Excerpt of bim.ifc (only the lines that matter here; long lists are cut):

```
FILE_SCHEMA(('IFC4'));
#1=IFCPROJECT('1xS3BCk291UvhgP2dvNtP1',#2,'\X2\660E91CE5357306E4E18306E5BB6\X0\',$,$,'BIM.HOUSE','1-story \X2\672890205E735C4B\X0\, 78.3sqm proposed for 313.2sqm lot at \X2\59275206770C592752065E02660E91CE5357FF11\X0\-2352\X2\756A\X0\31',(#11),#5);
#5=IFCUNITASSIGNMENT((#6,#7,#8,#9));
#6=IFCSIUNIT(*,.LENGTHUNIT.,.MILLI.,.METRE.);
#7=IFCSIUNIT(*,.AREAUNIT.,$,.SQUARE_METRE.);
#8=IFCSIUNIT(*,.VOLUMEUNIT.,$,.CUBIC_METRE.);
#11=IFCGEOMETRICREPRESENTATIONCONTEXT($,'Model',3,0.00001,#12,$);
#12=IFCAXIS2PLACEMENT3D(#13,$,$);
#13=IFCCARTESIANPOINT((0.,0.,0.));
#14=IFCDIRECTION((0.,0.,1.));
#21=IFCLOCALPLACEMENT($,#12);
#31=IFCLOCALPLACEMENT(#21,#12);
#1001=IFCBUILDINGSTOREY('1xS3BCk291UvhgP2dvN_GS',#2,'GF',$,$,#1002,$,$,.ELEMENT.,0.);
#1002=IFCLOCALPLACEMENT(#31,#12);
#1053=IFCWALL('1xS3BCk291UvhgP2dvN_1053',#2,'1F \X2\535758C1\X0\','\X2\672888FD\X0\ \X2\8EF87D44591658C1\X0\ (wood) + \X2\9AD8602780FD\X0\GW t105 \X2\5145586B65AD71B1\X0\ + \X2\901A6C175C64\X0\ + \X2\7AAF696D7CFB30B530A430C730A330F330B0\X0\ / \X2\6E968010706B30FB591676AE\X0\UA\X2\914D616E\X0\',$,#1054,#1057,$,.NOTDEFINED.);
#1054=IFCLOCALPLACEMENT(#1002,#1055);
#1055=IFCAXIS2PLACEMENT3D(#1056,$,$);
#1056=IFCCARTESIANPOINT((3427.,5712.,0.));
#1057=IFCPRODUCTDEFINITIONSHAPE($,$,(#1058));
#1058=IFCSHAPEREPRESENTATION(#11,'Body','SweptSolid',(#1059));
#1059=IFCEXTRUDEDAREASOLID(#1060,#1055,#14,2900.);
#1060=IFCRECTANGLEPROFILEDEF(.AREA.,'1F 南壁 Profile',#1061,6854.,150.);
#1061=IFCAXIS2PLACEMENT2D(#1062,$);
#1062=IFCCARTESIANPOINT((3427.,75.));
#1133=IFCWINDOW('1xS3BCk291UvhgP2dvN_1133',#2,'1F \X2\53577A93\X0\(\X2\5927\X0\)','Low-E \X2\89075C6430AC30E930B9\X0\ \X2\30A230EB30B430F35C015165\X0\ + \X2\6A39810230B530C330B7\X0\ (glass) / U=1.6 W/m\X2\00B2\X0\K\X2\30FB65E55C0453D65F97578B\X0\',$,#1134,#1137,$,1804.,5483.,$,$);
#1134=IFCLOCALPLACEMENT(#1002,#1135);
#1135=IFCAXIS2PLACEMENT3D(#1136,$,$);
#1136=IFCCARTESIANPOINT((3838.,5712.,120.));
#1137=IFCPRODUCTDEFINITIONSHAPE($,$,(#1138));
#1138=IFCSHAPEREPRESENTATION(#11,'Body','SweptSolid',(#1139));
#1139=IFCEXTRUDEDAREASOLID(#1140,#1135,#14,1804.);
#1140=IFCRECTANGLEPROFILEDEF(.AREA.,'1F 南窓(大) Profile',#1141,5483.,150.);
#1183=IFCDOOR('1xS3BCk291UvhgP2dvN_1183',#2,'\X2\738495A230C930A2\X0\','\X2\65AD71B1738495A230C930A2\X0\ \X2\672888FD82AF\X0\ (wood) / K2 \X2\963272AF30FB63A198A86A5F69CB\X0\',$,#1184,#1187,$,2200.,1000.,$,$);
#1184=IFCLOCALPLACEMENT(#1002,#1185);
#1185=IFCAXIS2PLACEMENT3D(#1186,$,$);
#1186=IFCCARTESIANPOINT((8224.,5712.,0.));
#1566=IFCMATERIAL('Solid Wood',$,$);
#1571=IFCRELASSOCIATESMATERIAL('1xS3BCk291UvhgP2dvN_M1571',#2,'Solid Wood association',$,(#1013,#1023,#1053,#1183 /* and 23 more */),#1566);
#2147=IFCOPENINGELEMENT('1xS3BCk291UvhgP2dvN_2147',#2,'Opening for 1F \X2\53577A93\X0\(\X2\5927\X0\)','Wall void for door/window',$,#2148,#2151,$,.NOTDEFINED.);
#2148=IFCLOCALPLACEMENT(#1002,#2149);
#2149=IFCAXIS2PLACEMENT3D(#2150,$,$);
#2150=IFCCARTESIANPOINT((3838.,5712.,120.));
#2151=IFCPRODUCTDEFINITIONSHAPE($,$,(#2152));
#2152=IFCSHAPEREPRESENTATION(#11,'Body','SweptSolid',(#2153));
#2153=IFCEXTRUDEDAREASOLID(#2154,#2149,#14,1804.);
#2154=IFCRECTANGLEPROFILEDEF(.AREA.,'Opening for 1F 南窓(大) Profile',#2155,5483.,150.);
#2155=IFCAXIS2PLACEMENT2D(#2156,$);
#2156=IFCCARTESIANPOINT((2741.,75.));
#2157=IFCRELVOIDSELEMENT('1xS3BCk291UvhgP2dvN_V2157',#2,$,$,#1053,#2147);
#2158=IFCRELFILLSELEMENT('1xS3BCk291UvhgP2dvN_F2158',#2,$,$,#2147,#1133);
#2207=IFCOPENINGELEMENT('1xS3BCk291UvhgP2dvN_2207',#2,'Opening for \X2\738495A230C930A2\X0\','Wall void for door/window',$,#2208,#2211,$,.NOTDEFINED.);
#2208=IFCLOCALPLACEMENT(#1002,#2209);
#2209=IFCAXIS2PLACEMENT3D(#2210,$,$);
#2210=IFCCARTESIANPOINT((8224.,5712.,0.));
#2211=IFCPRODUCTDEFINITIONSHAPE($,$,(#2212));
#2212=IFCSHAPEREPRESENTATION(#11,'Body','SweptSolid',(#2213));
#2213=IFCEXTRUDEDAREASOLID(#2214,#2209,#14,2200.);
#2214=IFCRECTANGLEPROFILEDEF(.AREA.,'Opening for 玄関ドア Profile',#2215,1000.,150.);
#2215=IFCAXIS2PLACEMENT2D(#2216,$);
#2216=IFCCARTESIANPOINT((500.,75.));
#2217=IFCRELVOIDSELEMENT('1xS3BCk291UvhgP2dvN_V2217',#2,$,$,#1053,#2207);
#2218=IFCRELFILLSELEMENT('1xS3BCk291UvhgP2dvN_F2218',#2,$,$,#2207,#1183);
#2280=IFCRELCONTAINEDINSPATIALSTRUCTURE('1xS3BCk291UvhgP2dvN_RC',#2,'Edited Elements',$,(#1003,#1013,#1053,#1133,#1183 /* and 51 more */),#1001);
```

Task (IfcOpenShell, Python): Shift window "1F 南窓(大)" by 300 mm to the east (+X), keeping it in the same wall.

```python
import ifcopenshell
import ifcopenshell.api.geometry
import ifcopenshell.util.placement
import ifcopenshell.util.unit

model = ifcopenshell.open("bim.ifc")
unit_scale = ifcopenshell.util.unit.calculate_unit_scale(model)

window = model.by_guid("1xS3BCk291UvhgP2dvN_1133")
opening = window.FillsVoids[0].RelatingOpeningElement
wall = opening.VoidsElements[0].RelatingBuildingElement

wall_matrix = ifcopenshell.util.placement.get_local_placement(wall.ObjectPlacement)
shift = wall_matrix[:3, 0] * 0.3 / unit_scale
before = ifcopenshell.util.placement.get_local_placement(window.ObjectPlacement)[:3, 3].copy()

# The window is not placed relative to its opening, so move both.
for product in (opening, window):
    matrix = ifcopenshell.util.placement.get_local_placement(product.ObjectPlacement)
    matrix[:3, 3] += shift
    ifcopenshell.api.geometry.edit_object_placement(model, product=product, matrix=matrix, is_si=False)

after = ifcopenshell.util.placement.get_local_placement(window.ObjectPlacement)[:3, 3]
print("window moved by", (after - before).round(3) + 0.0)

model.write("bim_edited.ifc")
```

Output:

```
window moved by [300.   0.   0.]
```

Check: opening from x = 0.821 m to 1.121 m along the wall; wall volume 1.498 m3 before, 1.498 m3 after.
